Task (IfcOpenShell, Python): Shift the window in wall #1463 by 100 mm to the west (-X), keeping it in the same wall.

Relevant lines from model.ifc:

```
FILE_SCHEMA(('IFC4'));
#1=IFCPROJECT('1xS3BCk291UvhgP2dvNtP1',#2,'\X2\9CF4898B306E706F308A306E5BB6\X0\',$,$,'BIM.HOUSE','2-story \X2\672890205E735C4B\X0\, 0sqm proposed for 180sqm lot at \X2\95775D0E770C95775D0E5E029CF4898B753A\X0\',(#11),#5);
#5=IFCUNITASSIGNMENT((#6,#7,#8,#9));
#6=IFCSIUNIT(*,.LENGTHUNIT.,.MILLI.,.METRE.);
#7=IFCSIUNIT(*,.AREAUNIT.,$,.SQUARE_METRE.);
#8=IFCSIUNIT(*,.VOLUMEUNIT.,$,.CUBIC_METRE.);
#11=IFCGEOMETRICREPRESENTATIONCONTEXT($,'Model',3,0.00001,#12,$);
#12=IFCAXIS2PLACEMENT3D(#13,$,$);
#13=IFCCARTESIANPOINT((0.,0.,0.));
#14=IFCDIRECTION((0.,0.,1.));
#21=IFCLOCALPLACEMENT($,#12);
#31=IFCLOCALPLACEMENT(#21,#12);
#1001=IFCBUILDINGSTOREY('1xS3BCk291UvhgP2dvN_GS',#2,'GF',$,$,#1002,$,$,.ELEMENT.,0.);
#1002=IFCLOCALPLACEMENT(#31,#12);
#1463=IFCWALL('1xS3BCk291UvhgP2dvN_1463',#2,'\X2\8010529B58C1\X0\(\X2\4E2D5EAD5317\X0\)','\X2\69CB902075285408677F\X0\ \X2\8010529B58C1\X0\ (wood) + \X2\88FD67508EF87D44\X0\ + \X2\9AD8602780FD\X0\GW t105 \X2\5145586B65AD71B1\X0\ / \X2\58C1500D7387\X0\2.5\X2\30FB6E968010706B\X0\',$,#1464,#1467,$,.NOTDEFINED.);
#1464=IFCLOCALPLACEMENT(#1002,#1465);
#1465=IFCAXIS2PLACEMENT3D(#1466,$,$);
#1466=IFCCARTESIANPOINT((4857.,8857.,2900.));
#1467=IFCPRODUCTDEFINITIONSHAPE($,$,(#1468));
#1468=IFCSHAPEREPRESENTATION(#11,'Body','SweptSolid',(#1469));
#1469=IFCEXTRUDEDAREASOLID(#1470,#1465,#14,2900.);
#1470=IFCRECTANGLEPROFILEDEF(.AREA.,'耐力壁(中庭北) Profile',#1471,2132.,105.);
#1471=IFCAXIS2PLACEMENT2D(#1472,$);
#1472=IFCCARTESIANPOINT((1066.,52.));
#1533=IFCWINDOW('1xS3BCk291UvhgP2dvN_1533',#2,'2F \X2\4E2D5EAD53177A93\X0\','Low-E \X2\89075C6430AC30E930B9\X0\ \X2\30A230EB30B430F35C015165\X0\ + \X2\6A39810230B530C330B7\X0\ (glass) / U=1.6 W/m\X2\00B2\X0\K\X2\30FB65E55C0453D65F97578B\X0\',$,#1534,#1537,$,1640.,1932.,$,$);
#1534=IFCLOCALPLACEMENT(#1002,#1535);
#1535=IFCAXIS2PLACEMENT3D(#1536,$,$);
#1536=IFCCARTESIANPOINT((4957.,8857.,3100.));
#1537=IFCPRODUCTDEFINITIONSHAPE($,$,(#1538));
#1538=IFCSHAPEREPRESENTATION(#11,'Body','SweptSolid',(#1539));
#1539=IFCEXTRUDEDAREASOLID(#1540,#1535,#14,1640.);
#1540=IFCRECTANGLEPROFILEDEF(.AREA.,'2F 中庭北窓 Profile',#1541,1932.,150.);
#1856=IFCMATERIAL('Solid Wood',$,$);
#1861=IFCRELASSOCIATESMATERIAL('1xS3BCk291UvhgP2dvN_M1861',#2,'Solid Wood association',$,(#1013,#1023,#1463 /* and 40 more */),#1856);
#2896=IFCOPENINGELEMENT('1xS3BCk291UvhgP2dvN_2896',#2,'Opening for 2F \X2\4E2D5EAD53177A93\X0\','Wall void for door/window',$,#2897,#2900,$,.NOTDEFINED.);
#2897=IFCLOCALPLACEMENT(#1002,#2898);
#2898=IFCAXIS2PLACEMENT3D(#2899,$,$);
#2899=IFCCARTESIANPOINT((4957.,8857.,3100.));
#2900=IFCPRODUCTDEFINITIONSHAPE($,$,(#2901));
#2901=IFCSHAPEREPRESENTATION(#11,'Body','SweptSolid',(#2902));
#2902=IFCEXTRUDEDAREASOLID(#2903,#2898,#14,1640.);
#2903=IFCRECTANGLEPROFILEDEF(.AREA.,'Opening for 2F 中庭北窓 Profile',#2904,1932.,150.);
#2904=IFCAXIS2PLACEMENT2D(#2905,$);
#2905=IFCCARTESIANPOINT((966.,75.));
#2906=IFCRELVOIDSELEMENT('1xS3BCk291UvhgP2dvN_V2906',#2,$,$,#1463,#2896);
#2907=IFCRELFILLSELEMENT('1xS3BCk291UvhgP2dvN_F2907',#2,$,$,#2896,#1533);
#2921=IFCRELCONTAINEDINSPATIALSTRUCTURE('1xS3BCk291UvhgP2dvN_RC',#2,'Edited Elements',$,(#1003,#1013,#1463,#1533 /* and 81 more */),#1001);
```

```python
import ifcopenshell
import ifcopenshell.api.geometry
import ifcopenshell.util.placement

model = ifcopenshell.open("model.ifc")

window = model.by_id(1533)
opening = window.FillsVoids[0].RelatingOpeningElement
wall = opening.VoidsElements[0].RelatingBuildingElement

wall_matrix = ifcopenshell.util.placement.get_local_placement(wall.ObjectPlacement)
shift = wall_matrix[:3, 0] * -100.0
before = ifcopenshell.util.placement.get_local_placement(window.ObjectPlacement)[:3, 3].copy()

# The window is not placed relative to its opening, so move both.
for product in (opening, window):
    matrix = ifcopenshell.util.placement.get_local_placement(product.ObjectPlacement)
    matrix[:3, 3] += shift
    ifcopenshell.api.geometry.edit_object_placement(model, product=product, matrix=matrix, is_si=False)

after = ifcopenshell.util.placement.get_local_placement(window.ObjectPlacement)[:3, 3]
print("window moved by", (after - before).round(3) + 0.0)

model.write("model_updated.ifc")
```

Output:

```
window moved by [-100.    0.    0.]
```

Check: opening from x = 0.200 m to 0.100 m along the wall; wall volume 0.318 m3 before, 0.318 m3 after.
